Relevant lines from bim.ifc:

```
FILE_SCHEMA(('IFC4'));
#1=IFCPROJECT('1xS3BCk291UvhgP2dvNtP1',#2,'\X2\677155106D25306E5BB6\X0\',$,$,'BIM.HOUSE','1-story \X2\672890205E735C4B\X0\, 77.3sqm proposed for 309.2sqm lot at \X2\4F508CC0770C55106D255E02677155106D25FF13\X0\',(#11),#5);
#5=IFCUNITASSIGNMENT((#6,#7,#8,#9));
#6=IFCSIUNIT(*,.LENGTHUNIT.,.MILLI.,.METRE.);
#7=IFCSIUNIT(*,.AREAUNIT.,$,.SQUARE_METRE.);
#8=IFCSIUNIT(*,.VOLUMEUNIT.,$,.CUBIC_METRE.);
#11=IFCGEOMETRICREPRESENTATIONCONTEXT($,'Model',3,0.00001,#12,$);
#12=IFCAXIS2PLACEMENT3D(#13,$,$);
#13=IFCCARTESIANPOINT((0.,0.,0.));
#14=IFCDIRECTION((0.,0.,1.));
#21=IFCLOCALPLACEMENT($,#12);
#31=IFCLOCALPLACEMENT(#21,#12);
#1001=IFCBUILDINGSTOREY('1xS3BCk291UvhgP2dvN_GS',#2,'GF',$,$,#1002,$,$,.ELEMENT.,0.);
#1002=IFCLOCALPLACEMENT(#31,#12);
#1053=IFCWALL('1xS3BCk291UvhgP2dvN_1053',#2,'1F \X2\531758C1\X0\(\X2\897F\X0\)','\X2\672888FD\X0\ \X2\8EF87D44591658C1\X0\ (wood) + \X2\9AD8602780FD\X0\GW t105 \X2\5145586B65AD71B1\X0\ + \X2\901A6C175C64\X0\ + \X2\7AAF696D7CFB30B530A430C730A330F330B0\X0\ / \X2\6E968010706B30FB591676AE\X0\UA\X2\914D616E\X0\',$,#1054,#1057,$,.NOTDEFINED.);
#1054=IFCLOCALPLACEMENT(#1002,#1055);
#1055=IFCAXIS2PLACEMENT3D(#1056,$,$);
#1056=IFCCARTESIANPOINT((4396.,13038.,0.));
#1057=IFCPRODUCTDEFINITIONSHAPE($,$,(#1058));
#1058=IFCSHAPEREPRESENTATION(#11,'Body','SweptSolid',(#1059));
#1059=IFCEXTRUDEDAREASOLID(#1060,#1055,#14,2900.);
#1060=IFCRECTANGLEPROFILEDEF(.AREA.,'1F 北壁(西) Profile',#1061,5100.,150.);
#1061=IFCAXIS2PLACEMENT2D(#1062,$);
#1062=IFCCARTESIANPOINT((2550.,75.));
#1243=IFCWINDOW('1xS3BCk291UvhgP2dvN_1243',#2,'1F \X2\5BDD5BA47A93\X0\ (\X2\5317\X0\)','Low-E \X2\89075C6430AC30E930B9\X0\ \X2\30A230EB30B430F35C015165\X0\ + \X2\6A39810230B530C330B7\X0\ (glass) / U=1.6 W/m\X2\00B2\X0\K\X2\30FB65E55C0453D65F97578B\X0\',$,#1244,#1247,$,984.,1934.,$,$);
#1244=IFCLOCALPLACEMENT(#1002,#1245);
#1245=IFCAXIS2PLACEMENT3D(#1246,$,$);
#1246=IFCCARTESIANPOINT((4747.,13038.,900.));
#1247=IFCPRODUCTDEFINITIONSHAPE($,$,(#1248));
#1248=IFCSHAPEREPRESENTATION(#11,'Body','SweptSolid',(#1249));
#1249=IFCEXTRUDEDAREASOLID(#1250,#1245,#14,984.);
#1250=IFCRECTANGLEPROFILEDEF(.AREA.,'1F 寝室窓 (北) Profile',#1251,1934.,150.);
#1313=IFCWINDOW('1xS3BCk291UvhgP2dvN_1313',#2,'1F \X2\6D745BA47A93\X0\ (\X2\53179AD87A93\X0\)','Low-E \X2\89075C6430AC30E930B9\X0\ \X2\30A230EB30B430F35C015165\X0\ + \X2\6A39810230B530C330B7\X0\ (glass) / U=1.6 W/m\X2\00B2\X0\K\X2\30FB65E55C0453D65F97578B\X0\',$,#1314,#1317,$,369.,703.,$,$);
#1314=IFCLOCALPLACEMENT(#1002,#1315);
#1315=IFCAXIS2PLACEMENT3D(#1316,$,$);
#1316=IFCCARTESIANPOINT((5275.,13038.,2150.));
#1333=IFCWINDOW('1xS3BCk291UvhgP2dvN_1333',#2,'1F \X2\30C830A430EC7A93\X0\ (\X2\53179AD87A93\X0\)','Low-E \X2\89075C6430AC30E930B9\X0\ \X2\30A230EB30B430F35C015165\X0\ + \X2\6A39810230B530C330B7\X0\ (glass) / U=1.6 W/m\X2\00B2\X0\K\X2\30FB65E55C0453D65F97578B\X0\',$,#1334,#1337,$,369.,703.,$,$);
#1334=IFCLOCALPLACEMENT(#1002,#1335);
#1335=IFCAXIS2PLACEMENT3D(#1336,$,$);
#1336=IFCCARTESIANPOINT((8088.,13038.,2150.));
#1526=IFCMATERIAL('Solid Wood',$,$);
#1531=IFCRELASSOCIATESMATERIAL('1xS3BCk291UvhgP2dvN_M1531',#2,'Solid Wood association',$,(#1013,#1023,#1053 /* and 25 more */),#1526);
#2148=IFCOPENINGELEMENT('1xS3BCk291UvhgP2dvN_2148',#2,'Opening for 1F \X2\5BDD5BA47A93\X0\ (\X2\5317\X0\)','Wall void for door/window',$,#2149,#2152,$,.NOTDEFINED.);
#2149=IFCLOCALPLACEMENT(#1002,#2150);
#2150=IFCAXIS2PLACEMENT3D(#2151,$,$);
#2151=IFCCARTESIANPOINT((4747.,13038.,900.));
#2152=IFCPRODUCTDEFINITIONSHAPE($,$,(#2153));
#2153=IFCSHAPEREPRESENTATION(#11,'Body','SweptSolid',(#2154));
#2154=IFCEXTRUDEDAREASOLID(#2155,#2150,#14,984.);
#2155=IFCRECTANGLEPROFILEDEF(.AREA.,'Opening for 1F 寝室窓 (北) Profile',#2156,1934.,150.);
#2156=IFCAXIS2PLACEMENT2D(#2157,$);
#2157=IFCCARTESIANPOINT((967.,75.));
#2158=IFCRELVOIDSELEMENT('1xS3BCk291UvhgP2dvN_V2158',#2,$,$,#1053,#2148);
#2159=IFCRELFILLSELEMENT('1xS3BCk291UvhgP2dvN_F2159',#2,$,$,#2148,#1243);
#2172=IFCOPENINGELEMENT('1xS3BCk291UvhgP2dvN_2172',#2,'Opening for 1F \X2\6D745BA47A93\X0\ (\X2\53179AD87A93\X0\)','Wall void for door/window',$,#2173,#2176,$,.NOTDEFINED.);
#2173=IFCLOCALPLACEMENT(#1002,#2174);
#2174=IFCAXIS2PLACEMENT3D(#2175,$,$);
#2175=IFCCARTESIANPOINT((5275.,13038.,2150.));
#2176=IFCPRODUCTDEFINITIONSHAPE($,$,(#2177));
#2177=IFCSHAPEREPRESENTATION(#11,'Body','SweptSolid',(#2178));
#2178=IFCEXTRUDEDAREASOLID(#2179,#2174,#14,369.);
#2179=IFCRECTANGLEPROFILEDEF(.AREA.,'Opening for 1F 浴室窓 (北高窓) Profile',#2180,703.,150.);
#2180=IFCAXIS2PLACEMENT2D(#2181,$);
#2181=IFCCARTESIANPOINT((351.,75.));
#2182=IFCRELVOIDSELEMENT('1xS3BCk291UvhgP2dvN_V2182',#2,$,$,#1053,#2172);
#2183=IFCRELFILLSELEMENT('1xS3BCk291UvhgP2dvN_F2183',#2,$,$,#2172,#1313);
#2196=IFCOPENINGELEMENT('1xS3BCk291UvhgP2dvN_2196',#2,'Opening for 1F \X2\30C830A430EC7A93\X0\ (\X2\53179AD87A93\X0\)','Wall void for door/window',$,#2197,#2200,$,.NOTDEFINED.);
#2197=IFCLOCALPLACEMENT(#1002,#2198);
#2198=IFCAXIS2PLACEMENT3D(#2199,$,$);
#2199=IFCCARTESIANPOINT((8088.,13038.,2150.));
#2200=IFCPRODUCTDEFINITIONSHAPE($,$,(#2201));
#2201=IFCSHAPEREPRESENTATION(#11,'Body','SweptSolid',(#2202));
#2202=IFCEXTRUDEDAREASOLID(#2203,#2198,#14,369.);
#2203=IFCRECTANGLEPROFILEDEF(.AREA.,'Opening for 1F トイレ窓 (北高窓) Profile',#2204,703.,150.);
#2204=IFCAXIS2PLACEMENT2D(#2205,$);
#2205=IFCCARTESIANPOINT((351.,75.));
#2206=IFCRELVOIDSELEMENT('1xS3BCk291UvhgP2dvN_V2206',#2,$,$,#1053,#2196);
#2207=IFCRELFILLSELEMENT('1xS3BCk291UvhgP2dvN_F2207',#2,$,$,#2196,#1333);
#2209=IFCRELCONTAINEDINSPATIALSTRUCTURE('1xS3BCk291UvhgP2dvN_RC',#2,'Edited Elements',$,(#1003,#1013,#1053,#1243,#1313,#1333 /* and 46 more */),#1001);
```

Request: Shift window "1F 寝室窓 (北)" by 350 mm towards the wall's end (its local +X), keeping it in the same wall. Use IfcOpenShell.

```python
import ifcopenshell
import ifcopenshell.api.geometry
import ifcopenshell.util.placement
import ifcopenshell.util.unit

model = ifcopenshell.open("bim.ifc")
unit_scale = ifcopenshell.util.unit.calculate_unit_scale(model)

window = model.by_id(1243)
opening = window.FillsVoids[0].RelatingOpeningElement
wall = opening.VoidsElements[0].RelatingBuildingElement

wall_matrix = ifcopenshell.util.placement.get_local_placement(wall.ObjectPlacement)
shift = wall_matrix[:3, 0] * 0.35 / unit_scale
before = ifcopenshell.util.placement.get_local_placement(window.ObjectPlacement)[:3, 3].copy()

# The window is not placed relative to its opening, so move both.
for product in (opening, window):
    matrix = ifcopenshell.util.placement.get_local_placement(product.ObjectPlacement)
    matrix[:3, 3] += shift
    ifcopenshell.api.geometry.edit_object_placement(model, product=product, matrix=matrix, is_si=False)

after = ifcopenshell.util.placement.get_local_placement(window.ObjectPlacement)[:3, 3]
print("window moved by", (after - before).round(3) + 0.0)

model.write("bim_updated.ifc")
```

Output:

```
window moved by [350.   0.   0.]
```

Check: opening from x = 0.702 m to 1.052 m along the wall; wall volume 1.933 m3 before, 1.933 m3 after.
